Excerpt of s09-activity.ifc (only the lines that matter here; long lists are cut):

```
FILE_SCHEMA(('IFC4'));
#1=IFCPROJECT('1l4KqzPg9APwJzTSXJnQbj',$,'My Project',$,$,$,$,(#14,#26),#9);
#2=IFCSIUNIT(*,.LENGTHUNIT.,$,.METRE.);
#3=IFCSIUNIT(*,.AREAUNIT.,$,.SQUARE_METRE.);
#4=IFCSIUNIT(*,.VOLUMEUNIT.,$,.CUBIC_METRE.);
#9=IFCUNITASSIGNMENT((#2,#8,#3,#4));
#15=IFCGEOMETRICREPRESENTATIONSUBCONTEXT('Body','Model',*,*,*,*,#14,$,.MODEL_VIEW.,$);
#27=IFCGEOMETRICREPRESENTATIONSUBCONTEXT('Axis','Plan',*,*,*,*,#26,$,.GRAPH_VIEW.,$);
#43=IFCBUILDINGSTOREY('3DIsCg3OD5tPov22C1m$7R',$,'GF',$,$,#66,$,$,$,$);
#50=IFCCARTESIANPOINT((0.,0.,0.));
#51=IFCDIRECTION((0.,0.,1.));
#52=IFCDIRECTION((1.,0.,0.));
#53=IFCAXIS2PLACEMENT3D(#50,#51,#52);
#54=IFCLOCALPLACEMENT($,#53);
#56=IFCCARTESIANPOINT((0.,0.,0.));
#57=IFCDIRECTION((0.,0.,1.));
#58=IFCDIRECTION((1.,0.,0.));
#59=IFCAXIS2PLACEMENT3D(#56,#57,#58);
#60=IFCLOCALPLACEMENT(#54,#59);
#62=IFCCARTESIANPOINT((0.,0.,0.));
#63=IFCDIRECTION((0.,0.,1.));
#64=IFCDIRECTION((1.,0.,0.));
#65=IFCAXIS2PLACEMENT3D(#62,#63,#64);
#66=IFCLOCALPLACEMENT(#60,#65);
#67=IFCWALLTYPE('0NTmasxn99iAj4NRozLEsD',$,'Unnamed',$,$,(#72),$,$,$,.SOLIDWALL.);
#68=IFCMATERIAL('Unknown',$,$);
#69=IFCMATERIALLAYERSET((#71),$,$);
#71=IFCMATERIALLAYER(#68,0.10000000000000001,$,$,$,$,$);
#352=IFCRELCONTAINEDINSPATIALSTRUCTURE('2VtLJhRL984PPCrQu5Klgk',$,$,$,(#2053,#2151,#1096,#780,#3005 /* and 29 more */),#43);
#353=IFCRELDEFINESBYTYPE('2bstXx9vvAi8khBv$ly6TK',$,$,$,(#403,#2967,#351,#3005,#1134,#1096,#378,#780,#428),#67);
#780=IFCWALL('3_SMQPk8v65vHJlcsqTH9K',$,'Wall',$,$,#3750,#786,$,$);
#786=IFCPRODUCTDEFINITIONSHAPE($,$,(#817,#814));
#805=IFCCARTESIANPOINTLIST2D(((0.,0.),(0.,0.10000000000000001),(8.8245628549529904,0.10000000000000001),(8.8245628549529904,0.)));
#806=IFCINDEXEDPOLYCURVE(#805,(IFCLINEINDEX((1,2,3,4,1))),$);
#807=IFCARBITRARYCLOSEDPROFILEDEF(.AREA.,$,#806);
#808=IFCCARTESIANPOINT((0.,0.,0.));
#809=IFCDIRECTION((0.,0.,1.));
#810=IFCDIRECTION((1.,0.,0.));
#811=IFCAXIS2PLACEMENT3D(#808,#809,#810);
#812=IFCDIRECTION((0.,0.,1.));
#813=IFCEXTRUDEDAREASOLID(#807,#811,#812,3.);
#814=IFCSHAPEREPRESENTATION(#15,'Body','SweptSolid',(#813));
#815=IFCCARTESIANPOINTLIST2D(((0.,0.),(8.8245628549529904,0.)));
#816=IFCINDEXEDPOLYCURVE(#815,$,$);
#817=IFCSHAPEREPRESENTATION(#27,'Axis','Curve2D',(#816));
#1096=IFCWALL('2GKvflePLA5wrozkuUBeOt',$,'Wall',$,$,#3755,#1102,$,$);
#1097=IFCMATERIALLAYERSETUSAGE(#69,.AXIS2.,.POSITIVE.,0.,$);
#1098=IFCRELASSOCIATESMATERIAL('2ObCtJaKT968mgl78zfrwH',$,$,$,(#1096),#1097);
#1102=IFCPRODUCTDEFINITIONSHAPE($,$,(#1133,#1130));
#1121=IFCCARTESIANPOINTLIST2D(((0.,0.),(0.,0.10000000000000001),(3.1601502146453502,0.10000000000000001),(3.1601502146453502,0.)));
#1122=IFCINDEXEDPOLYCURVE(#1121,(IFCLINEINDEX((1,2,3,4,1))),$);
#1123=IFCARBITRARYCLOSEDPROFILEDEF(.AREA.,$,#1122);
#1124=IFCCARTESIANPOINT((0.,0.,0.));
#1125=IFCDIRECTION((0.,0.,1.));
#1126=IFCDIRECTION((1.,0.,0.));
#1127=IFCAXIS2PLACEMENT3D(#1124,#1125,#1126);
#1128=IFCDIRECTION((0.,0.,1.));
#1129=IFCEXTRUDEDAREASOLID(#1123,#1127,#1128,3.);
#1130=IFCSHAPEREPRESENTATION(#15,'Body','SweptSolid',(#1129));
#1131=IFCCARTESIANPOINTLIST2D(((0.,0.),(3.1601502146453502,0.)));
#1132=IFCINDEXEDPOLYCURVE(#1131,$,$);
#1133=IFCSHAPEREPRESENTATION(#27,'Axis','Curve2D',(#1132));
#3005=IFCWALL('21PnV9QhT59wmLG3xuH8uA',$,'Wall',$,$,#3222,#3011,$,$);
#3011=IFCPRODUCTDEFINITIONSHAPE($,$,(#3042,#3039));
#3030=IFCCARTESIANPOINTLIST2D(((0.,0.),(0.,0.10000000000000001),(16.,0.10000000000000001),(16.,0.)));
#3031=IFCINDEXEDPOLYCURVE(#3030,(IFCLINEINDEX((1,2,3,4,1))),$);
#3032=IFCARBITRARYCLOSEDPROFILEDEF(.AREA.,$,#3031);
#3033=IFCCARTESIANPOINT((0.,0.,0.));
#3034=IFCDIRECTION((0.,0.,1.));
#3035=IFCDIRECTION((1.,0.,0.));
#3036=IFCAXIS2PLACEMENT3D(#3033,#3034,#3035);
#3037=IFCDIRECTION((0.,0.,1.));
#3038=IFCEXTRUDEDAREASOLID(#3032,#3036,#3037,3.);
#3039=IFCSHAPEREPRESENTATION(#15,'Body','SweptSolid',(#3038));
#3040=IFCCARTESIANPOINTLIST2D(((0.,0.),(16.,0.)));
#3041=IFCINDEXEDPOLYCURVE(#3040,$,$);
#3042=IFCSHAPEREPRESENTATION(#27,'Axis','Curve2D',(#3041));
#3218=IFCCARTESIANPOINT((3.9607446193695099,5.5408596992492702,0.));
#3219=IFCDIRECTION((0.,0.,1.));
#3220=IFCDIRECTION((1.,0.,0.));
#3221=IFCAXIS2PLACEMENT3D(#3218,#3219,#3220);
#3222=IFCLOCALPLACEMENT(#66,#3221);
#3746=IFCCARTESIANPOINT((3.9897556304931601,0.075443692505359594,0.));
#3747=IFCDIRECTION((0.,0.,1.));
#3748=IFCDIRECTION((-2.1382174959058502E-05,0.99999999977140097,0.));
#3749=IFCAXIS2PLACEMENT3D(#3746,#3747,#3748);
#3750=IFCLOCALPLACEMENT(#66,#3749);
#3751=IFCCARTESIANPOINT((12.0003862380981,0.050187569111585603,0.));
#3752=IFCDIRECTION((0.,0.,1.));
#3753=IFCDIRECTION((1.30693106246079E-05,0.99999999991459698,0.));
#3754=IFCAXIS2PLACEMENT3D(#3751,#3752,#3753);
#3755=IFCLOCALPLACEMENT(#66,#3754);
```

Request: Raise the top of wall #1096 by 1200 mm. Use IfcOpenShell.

```python
import ifcopenshell
import ifcopenshell.geom
import ifcopenshell.util.representation
import ifcopenshell.util.shape
import ifcopenshell.util.unit

model = ifcopenshell.open("s09-activity.ifc")
unit_scale = ifcopenshell.util.unit.calculate_unit_scale(model)
settings = ifcopenshell.geom.settings()


def volume(element):
    """Net volume in cubic metres, openings subtracted."""
    shape = ifcopenshell.geom.create_shape(settings, element)
    return ifcopenshell.util.shape.get_volume(shape.geometry)


wall = model.by_id(1096)
before = volume(wall)

body = ifcopenshell.util.representation.get_representation(wall, "Model", "Body")
solid = body.Items[0]
old_height = solid.Depth
solid.Depth += 1.2 / unit_scale
after = volume(wall)

print(f"height {old_height:g} -> {solid.Depth:g}, volume {before:.3f} -> {after:.3f} m3")

model.write("s09-activity_rev.ifc")
```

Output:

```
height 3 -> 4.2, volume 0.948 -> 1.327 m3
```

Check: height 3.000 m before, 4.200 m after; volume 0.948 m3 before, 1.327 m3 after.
